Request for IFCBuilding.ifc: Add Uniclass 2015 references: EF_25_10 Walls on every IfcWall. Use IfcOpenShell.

First a look at what the model holds.

```python
import ifcopenshell

model = ifcopenshell.open("IFCBuilding.ifc")
print(model.schema)
print("classifications:", [c.Name for c in model.by_type("IfcClassification")])
for ifc_class in ("IfcDoor", "IfcRoof", "IfcStair", "IfcWall", "IfcWindow"):
    print(ifc_class, len(model.by_type(ifc_class)))
```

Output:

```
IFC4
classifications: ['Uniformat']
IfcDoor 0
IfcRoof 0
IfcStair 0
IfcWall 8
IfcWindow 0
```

```python
import ifcopenshell
import ifcopenshell.api.classification

model = ifcopenshell.open("IFCBuilding.ifc")

system = ifcopenshell.api.classification.add_classification(model, classification="Uniclass 2015")

codes = {
    "IfcWall": ("EF_25_10", "Walls"),
}
for ifc_class, (code, name) in codes.items():
    products = model.by_type(ifc_class)
    ifcopenshell.api.classification.add_reference(
        model, products=products, classification=system, identification=code, name=name
    )
    print(code, len(products))

model.write("IFCBuilding_rev.ifc")
```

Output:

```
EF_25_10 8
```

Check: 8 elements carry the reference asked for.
